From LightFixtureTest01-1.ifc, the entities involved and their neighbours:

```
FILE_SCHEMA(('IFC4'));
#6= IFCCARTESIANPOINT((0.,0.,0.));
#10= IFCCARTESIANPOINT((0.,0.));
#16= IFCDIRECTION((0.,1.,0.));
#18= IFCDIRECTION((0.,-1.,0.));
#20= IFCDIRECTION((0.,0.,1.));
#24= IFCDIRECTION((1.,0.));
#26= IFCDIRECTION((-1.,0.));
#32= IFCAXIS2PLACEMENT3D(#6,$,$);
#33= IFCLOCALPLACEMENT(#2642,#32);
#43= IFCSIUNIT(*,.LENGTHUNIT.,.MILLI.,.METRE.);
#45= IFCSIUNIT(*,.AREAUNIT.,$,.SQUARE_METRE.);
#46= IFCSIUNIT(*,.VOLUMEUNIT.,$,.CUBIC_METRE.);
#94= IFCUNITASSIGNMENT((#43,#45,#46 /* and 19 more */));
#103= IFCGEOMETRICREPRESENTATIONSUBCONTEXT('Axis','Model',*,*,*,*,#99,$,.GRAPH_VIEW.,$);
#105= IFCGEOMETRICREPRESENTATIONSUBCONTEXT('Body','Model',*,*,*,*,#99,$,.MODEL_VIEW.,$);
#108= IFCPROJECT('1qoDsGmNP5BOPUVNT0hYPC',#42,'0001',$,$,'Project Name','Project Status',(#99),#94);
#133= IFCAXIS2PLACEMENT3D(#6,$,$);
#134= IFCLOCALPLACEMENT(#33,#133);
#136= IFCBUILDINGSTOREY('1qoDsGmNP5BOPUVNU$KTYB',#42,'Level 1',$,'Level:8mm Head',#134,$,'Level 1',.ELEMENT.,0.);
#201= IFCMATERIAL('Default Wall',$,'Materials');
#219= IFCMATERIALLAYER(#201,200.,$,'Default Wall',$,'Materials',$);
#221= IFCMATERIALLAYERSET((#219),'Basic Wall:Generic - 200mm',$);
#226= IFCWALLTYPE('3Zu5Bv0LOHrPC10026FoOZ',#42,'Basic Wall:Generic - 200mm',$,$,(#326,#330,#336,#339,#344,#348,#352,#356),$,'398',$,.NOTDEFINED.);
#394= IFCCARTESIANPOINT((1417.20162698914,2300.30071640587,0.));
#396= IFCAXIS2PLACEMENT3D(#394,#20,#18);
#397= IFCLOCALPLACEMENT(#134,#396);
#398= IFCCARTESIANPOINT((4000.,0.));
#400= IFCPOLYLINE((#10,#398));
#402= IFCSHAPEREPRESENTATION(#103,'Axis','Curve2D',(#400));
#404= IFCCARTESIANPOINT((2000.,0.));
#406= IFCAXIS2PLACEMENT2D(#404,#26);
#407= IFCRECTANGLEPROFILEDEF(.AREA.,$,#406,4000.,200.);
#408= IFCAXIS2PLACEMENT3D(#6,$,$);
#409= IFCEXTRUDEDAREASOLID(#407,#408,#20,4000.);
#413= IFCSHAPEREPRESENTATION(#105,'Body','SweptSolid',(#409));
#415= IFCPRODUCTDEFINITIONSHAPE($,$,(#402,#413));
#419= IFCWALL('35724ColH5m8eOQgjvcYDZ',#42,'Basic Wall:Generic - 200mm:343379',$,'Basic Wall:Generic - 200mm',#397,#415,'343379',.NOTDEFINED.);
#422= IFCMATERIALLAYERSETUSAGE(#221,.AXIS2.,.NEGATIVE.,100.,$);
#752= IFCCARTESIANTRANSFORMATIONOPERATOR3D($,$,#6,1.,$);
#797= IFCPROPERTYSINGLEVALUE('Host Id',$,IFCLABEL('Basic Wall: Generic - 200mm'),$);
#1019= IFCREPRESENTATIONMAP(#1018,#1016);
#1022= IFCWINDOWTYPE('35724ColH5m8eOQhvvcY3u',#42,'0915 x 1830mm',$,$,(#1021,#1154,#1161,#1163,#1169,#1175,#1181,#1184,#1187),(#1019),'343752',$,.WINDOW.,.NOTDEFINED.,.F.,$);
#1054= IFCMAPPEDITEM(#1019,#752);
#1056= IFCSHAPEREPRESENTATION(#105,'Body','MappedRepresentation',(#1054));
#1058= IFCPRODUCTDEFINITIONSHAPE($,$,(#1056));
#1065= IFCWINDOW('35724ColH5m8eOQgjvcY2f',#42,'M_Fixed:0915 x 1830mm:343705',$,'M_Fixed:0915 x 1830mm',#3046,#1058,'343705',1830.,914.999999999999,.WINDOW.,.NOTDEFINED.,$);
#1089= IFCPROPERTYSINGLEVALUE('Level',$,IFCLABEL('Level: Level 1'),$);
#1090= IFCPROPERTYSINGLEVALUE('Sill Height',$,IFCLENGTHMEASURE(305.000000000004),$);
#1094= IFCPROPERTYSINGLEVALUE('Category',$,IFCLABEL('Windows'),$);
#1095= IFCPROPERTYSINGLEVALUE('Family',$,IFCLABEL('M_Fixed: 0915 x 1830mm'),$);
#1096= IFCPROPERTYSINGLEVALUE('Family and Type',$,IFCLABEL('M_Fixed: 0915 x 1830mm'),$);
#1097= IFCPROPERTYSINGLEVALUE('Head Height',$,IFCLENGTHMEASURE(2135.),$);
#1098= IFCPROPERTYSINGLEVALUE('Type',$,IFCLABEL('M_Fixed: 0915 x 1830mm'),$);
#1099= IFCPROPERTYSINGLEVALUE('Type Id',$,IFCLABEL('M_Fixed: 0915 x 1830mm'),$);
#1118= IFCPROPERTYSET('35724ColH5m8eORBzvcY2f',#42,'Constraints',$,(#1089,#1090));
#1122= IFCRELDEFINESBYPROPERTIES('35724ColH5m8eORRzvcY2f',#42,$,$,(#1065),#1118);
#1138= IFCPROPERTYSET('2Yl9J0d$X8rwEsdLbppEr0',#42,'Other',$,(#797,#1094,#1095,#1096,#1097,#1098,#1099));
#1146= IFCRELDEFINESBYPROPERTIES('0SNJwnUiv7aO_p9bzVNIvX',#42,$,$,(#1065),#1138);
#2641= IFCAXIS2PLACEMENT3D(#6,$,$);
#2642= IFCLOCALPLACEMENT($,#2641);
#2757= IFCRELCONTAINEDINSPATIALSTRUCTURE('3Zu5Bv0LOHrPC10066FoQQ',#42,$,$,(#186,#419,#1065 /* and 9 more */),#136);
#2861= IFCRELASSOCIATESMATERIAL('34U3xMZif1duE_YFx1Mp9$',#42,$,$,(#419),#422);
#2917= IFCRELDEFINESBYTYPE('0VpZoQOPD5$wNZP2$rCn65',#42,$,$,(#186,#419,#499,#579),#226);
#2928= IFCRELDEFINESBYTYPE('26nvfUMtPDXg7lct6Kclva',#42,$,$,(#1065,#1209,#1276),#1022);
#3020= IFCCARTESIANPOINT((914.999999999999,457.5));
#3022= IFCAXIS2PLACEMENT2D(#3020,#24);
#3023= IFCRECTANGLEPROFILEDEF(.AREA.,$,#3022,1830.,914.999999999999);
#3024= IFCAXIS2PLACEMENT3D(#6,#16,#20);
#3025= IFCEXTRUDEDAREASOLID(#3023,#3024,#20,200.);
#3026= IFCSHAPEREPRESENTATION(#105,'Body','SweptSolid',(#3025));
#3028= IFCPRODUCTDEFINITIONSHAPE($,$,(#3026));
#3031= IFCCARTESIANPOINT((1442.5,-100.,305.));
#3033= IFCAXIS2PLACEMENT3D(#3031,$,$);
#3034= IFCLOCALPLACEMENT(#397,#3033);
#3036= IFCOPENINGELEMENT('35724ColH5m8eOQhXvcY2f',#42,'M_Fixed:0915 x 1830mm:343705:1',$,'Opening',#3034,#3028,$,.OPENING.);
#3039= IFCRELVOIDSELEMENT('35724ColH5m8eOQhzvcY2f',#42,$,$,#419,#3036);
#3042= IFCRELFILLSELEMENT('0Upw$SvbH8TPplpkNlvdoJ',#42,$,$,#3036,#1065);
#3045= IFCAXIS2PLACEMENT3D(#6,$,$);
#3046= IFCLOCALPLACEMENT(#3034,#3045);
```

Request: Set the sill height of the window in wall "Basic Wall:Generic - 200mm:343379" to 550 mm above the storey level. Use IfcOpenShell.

```python
import numpy as np
import ifcopenshell
import ifcopenshell.api.geometry
import ifcopenshell.api.pset
import ifcopenshell.geom
import ifcopenshell.util.element
import ifcopenshell.util.placement
import ifcopenshell.util.shape
import ifcopenshell.util.unit

model = ifcopenshell.open("LightFixtureTest01-1.ifc")
unit_scale = ifcopenshell.util.unit.calculate_unit_scale(model)

window = model.by_guid("35724ColH5m8eOQgjvcY2f")
opening = window.FillsVoids[0].RelatingOpeningElement
storey = ifcopenshell.util.element.get_container(window, ifc_class="IfcBuildingStorey")
level = ifcopenshell.util.placement.get_local_placement(storey.ObjectPlacement)[2, 3]

# The opening's origin need not be at the sill, so measure its lowest point.
shape = ifcopenshell.geom.create_shape(ifcopenshell.geom.settings(), opening)
bottom = ifcopenshell.util.shape.get_shape_bottom_elevation(shape, shape.geometry) / unit_scale
dz = level + 550.0 - bottom

shift = np.array([0.0, 0.0, dz])
# The window is placed relative to its opening, so it follows when the opening moves.
matrix = ifcopenshell.util.placement.get_local_placement(opening.ObjectPlacement)
matrix[:3, 3] += shift
ifcopenshell.api.geometry.edit_object_placement(
    model, product=opening, matrix=matrix, is_si=False, should_transform_children=True
)

# Keep the stored heights in step.
pset = model.by_id(ifcopenshell.util.element.get_pset(window, "Constraints", should_inherit=False)["id"])
ifcopenshell.api.pset.edit_pset(model, pset=pset, properties={
    "Sill Height": model.create_entity("IfcLengthMeasure", ifcopenshell.util.element.get_pset(window, "Constraints", "Sill Height") + dz),
})
pset = model.by_id(ifcopenshell.util.element.get_pset(window, "Other", should_inherit=False)["id"])
ifcopenshell.api.pset.edit_pset(model, pset=pset, properties={
    "Head Height": model.create_entity("IfcLengthMeasure", ifcopenshell.util.element.get_pset(window, "Other", "Head Height") + dz),
})

print(f"moved by {dz * unit_scale:+.3f} m")

model.write("LightFixtureTest01-1_updated.ifc")
```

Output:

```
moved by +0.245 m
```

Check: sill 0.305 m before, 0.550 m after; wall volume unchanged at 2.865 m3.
